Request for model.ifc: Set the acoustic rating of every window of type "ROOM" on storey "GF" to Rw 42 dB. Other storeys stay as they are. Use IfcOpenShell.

First a look at what the model holds.

```python
import ifcopenshell
import ifcopenshell.util.element

model = ifcopenshell.open("model.ifc")
print(model.schema)
storey = next(s for s in model.by_type("IfcBuildingStorey") if s.Name == "GF")
windows = [e for e in ifcopenshell.util.element.get_decomposition(storey) if e.is_a("IfcWindow")]
seen = {}
for e in windows:
    element_type = ifcopenshell.util.element.get_type(e)
    key = (element_type.Name if element_type != e and element_type else None, ifcopenshell.util.element.get_pset(e, "Pset_WindowCommon", "AcousticRating"))
    seen[key] = seen.get(key, 0) + 1
for (name, value), count in sorted(seen.items(), key=str):
    print(count, "x", name, "|", value)
```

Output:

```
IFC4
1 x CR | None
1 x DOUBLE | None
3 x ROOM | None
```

```python
import ifcopenshell
import ifcopenshell.api.pset
import ifcopenshell.util.element

model = ifcopenshell.open("model.ifc")

storey = next(s for s in model.by_type("IfcBuildingStorey") if s.Name == "GF")
windows = [e for e in ifcopenshell.util.element.get_decomposition(storey) if e.is_a("IfcWindow")]

count = 0
for e in windows:
    element_type = ifcopenshell.util.element.get_type(e)
    if element_type in (None, e) or element_type.Name != "ROOM":
        continue
    # add_pset returns the element's existing set when there is one.
    pset = ifcopenshell.api.pset.add_pset(model, product=e, name="Pset_WindowCommon")
    ifcopenshell.api.pset.edit_pset(model, pset=pset, properties={"AcousticRating": "Rw 42 dB"})
    count += 1

print(count, "windows updated")

model.write("model_updated.ifc")
```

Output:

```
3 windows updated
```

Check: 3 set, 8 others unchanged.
